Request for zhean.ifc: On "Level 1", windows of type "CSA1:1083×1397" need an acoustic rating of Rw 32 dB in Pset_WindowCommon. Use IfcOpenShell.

First a look at what the model holds.

```python
import ifcopenshell
import ifcopenshell.util.element

model = ifcopenshell.open("zhean.ifc")
print(model.schema)
storey = next(s for s in model.by_type("IfcBuildingStorey") if s.Name == "Level 1")
windows = [e for e in ifcopenshell.util.element.get_decomposition(storey) if e.is_a("IfcWindow")]
seen = {}
for e in windows:
    element_type = ifcopenshell.util.element.get_type(e)
    key = (element_type.Name if element_type != e and element_type else None, ifcopenshell.util.element.get_pset(e, "Pset_WindowCommon", "AcousticRating"))
    seen[key] = seen.get(key, 0) + 1
for (name, value), count in sorted(seen.items(), key=str):
    print(count, "x", name, "|", value)
```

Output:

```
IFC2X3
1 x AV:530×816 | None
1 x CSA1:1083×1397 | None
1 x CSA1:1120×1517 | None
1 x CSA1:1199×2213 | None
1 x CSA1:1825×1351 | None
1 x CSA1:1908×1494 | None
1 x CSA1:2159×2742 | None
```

```python
import ifcopenshell
import ifcopenshell.api.pset
import ifcopenshell.util.element

model = ifcopenshell.open("zhean.ifc")

storey = next(s for s in model.by_type("IfcBuildingStorey") if s.Name == "Level 1")
windows = [e for e in ifcopenshell.util.element.get_decomposition(storey) if e.is_a("IfcWindow")]

count = 0
for e in windows:
    element_type = ifcopenshell.util.element.get_type(e)
    if element_type in (None, e) or element_type.Name != "CSA1:1083×1397":
        continue
    # add_pset returns the element's existing set when there is one.
    pset = ifcopenshell.api.pset.add_pset(model, product=e, name="Pset_WindowCommon")
    ifcopenshell.api.pset.edit_pset(model, pset=pset, properties={"AcousticRating": "Rw 32 dB"})
    count += 1

print(count, "windows updated")

model.write("zhean_edited.ifc")
```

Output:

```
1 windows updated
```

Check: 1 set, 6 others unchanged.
